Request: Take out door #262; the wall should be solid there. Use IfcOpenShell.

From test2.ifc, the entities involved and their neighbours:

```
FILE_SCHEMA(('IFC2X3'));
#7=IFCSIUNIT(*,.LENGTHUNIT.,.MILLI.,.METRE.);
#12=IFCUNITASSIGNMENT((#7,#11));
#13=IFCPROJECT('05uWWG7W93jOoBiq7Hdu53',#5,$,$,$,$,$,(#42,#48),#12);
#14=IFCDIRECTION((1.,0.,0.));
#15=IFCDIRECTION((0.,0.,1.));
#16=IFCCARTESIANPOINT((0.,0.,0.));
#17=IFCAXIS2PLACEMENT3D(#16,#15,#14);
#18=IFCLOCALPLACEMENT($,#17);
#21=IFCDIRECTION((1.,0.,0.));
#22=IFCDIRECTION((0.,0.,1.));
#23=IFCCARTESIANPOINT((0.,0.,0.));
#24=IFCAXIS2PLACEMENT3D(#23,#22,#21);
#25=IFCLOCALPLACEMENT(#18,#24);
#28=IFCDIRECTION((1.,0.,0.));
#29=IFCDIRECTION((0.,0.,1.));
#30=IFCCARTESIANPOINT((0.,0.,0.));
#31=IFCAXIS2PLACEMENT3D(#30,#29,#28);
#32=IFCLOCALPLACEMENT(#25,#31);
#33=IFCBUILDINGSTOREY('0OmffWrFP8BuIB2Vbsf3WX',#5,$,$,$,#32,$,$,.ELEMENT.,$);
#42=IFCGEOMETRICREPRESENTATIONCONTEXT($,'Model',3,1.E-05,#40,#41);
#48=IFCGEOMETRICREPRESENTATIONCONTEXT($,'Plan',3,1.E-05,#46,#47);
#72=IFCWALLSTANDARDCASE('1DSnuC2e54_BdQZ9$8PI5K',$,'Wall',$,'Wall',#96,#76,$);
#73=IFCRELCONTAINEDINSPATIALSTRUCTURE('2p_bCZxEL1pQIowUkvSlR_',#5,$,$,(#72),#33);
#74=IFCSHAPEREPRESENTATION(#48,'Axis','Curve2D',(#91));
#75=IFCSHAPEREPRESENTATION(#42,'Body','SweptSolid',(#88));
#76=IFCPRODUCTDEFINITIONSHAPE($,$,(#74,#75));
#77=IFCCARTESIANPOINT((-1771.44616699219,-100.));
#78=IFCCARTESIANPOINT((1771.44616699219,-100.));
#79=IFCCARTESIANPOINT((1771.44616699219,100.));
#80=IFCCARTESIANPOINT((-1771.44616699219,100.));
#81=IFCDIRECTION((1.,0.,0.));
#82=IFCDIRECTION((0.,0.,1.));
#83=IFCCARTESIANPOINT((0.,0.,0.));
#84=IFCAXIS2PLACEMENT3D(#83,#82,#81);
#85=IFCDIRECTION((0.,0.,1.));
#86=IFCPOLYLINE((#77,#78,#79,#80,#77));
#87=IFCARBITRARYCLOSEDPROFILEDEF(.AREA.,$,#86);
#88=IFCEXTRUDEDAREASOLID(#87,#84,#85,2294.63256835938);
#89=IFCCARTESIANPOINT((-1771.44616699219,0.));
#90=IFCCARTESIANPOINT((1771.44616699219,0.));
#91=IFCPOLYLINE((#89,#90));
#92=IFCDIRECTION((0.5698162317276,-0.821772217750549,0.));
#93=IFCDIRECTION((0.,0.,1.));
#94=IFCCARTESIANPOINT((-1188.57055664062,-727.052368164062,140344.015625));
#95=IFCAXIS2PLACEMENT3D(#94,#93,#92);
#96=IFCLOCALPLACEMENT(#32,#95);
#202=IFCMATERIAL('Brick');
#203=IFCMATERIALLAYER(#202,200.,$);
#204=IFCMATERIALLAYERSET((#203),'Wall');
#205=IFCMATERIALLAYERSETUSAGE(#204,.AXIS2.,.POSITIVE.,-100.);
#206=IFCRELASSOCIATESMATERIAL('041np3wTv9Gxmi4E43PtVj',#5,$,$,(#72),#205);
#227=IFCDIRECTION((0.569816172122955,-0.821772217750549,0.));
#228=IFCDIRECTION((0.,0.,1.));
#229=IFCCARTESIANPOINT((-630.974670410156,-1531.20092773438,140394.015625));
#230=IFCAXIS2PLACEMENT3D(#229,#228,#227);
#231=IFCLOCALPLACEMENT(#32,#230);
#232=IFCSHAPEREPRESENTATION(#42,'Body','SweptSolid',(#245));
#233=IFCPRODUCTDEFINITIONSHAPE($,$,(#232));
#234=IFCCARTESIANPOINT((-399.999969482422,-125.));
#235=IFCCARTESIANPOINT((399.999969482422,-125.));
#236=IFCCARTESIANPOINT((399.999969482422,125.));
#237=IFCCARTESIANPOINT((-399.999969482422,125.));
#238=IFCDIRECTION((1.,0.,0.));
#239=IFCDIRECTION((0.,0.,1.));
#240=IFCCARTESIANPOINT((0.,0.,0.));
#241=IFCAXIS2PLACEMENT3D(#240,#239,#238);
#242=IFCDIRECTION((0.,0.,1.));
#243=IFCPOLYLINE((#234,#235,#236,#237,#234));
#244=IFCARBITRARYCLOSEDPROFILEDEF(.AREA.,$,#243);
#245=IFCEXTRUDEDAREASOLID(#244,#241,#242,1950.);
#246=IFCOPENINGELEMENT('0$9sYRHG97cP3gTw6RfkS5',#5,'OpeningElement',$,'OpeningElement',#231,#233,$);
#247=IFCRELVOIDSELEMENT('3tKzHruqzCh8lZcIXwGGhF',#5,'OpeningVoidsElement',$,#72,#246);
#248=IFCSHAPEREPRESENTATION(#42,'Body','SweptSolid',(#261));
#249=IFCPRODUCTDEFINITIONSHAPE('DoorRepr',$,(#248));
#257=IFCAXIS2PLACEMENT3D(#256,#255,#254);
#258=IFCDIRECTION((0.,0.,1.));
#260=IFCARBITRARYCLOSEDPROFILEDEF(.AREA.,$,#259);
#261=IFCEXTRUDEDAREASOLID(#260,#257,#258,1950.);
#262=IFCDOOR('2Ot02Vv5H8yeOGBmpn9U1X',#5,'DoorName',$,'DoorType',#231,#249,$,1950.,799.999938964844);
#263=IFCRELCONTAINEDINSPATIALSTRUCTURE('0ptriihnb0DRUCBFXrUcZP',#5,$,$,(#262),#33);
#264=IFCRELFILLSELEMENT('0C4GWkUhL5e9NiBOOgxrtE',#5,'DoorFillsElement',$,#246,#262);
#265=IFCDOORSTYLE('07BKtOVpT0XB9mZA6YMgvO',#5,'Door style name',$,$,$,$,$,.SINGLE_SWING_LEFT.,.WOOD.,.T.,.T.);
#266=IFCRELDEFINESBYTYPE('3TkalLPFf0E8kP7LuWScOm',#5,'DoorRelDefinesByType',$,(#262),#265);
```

```python
import ifcopenshell
import ifcopenshell.api.feature
import ifcopenshell.api.root
import ifcopenshell.geom
import ifcopenshell.util.shape

model = ifcopenshell.open("test2.ifc")
settings = ifcopenshell.geom.settings()


def volume(element):
    """Net volume in cubic metres, openings subtracted."""
    shape = ifcopenshell.geom.create_shape(settings, element)
    return ifcopenshell.util.shape.get_volume(shape.geometry)


door = model.by_guid("2Ot02Vv5H8yeOGBmpn9U1X")
opening = door.FillsVoids[0].RelatingOpeningElement
wall = opening.VoidsElements[0].RelatingBuildingElement
before = volume(wall)

ifcopenshell.api.root.remove_product(model, product=door)
ifcopenshell.api.feature.remove_feature(model, feature=opening)

after = volume(wall)

print(f"wall volume {before:.3f} -> {after:.3f} m3")

model.write("test2_rev.ifc")
```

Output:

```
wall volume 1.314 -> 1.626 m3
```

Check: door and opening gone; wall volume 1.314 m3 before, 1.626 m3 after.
